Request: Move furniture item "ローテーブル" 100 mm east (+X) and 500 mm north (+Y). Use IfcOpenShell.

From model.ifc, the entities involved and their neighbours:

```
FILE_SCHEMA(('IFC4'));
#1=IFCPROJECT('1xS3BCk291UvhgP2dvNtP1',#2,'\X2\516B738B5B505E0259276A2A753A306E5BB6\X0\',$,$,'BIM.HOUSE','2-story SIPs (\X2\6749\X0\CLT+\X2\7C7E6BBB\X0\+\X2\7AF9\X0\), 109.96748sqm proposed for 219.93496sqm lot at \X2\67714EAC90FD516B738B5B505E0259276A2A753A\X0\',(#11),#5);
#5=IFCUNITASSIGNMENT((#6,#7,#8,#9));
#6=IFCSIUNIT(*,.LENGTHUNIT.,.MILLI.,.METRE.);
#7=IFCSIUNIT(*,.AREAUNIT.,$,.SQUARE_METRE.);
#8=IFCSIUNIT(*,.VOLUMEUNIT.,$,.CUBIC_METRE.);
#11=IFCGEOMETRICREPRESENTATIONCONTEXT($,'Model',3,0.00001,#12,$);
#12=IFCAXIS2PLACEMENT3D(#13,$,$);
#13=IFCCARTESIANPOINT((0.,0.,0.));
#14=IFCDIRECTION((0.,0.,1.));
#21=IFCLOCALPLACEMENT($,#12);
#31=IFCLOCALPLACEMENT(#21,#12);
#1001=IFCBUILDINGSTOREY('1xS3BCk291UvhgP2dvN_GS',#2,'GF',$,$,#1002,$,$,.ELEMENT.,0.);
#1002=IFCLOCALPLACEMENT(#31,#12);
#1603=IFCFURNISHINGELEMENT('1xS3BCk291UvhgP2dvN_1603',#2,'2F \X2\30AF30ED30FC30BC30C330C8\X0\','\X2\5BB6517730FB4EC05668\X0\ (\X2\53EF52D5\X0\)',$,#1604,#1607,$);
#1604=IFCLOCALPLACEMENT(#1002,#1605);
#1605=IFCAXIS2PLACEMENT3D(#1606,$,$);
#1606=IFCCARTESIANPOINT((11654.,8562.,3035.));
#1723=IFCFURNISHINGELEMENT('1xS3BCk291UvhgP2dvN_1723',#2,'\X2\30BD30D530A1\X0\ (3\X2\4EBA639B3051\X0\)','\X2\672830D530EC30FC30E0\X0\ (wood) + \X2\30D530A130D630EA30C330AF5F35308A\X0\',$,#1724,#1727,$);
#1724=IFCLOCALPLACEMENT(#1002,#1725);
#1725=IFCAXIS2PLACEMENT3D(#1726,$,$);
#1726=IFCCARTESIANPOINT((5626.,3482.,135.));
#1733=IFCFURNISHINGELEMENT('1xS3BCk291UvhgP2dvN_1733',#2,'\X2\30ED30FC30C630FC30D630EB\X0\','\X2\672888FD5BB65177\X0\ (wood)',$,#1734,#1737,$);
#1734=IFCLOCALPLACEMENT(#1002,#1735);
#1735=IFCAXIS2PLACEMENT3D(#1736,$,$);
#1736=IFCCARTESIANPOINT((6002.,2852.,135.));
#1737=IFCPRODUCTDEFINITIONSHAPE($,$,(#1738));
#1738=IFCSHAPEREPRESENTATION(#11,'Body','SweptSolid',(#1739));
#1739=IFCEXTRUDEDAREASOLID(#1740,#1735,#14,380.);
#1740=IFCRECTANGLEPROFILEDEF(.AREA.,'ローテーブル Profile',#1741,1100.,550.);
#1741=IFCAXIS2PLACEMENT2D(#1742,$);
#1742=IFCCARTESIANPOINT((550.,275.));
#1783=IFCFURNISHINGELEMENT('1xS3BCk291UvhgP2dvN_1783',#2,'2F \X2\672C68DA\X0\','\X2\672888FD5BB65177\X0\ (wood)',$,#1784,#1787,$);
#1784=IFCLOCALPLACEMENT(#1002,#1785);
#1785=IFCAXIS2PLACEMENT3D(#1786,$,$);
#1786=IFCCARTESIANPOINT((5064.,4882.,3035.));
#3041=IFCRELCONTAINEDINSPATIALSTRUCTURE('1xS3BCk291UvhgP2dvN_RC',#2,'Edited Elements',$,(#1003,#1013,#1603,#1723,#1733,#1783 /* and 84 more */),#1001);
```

```python
import ifcopenshell
import ifcopenshell.api.geometry
import ifcopenshell.util.placement

model = ifcopenshell.open("model.ifc")

item = model.by_id(1733)
matrix = ifcopenshell.util.placement.get_local_placement(item.ObjectPlacement)
matrix[0, 3] += 100.0
matrix[1, 3] += 500.0
ifcopenshell.api.geometry.edit_object_placement(model, product=item, matrix=matrix, is_si=False)

print(ifcopenshell.util.placement.get_local_placement(item.ObjectPlacement).round(3) + 0.0)

model.write("model_rev.ifc")
```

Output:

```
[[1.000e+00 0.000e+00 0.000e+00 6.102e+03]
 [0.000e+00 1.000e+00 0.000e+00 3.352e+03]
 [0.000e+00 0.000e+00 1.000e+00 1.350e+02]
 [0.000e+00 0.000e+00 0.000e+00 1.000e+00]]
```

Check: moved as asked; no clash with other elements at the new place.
